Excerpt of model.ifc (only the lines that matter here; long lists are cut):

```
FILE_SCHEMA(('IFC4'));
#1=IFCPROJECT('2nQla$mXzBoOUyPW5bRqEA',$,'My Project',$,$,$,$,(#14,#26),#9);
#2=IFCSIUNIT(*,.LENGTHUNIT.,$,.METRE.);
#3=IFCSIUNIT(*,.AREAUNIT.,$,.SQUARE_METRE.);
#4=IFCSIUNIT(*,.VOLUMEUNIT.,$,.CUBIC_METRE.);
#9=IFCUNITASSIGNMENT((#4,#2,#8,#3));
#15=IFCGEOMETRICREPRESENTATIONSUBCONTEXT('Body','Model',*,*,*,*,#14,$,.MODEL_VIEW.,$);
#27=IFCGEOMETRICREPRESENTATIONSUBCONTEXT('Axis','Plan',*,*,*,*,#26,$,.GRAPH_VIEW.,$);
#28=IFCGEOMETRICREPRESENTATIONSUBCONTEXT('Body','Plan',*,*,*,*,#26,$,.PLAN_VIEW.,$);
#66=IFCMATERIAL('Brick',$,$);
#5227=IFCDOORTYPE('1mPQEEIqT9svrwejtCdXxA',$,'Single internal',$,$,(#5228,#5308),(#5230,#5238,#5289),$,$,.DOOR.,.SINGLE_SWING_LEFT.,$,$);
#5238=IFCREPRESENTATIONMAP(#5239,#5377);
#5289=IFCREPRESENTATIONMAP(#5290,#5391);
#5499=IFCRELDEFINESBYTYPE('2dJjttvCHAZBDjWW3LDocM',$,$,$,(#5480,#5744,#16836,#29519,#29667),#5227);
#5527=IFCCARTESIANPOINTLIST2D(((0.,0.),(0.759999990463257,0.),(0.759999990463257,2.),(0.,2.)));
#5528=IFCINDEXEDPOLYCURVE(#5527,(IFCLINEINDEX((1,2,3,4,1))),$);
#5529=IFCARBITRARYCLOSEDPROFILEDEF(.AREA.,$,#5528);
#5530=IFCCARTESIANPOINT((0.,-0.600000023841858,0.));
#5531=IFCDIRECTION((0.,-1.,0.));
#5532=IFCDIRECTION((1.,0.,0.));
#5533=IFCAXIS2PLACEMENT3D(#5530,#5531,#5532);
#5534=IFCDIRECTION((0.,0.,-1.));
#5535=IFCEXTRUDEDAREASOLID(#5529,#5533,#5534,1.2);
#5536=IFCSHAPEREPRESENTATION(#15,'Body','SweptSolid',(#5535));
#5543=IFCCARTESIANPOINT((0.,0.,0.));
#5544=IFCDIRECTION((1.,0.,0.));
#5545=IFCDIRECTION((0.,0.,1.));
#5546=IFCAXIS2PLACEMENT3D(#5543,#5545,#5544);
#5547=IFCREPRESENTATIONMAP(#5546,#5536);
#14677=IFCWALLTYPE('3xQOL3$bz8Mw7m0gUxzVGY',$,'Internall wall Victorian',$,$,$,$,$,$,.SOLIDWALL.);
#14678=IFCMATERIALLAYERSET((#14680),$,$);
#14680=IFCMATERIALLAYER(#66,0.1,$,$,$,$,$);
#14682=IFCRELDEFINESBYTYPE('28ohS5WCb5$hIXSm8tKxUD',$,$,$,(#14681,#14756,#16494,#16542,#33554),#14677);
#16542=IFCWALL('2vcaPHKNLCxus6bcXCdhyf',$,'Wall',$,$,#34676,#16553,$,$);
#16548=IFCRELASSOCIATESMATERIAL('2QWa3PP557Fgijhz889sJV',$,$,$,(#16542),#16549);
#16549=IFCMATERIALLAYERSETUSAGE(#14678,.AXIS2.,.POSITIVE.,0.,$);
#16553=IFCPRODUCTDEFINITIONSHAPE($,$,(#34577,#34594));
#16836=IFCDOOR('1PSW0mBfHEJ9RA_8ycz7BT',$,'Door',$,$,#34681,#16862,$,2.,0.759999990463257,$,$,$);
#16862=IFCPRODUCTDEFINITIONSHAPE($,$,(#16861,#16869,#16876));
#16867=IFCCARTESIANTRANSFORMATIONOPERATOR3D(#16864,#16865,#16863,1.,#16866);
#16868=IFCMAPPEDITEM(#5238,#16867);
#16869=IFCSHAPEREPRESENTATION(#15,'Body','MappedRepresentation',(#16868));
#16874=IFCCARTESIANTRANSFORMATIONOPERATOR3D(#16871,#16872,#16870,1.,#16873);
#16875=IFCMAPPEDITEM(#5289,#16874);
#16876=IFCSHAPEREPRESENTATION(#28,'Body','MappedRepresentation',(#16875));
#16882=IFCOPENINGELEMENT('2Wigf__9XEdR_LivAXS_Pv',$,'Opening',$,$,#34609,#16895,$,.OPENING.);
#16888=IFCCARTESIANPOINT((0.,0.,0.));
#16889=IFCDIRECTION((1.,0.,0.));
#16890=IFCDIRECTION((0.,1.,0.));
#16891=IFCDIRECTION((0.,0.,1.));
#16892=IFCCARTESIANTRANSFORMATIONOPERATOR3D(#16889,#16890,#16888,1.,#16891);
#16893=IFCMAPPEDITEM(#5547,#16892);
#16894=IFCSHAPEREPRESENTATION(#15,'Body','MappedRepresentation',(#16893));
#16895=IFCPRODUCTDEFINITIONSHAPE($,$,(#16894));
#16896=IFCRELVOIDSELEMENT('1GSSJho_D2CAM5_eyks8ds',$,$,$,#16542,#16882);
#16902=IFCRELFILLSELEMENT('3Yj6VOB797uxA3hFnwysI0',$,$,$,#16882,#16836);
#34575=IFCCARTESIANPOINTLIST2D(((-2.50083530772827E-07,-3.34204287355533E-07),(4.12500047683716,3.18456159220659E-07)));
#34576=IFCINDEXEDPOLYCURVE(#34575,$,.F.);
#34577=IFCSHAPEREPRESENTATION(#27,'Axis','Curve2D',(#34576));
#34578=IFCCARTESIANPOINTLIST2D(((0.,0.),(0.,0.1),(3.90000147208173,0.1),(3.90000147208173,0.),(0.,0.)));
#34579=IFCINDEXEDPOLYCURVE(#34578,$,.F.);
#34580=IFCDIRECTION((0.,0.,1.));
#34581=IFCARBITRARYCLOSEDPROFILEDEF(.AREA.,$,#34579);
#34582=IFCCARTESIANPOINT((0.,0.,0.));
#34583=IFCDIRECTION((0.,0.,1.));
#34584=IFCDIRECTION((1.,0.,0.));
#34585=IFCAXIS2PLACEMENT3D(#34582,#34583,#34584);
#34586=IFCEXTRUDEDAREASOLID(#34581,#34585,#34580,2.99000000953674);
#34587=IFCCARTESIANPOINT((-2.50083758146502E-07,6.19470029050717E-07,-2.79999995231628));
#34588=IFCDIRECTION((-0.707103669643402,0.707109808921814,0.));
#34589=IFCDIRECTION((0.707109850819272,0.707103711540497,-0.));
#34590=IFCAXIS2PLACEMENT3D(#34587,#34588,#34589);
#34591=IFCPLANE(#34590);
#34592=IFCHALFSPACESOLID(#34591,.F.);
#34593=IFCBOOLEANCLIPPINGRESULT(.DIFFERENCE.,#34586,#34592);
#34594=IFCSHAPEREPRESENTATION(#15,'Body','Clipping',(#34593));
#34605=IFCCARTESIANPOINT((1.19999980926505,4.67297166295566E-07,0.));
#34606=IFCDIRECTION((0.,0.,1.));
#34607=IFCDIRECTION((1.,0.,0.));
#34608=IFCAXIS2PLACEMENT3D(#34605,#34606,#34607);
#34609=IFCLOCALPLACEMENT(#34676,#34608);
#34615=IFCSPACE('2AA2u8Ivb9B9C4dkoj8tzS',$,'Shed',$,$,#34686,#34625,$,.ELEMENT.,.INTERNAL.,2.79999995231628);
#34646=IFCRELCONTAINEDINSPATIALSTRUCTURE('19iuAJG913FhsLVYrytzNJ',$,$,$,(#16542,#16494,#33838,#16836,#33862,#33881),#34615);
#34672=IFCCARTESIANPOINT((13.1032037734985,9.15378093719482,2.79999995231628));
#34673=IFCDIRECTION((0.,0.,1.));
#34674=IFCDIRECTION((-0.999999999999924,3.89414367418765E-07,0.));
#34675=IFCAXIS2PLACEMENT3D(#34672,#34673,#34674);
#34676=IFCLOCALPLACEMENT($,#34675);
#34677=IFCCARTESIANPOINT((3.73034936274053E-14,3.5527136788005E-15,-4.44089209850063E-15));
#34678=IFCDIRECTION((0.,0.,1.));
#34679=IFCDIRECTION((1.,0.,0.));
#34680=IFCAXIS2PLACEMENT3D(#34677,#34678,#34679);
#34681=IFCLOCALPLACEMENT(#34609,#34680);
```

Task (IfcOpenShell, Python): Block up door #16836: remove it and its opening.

```python
import ifcopenshell
import ifcopenshell.api.feature
import ifcopenshell.api.root
import ifcopenshell.geom
import ifcopenshell.util.shape

model = ifcopenshell.open("model.ifc")
settings = ifcopenshell.geom.settings()


def volume(element):
    """Net volume in cubic metres, openings subtracted."""
    shape = ifcopenshell.geom.create_shape(settings, element)
    return ifcopenshell.util.shape.get_volume(shape.geometry)


door = model.by_guid("1PSW0mBfHEJ9RA_8ycz7BT")
opening = door.FillsVoids[0].RelatingOpeningElement
wall = opening.VoidsElements[0].RelatingBuildingElement
before = volume(wall)

ifcopenshell.api.root.remove_product(model, product=door)
ifcopenshell.api.feature.remove_feature(model, feature=opening)

after = volume(wall)

print(f"wall volume {before:.3f} -> {after:.3f} m3")

model.write("model_edited.ifc")
```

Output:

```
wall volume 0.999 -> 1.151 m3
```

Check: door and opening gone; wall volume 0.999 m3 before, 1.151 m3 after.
